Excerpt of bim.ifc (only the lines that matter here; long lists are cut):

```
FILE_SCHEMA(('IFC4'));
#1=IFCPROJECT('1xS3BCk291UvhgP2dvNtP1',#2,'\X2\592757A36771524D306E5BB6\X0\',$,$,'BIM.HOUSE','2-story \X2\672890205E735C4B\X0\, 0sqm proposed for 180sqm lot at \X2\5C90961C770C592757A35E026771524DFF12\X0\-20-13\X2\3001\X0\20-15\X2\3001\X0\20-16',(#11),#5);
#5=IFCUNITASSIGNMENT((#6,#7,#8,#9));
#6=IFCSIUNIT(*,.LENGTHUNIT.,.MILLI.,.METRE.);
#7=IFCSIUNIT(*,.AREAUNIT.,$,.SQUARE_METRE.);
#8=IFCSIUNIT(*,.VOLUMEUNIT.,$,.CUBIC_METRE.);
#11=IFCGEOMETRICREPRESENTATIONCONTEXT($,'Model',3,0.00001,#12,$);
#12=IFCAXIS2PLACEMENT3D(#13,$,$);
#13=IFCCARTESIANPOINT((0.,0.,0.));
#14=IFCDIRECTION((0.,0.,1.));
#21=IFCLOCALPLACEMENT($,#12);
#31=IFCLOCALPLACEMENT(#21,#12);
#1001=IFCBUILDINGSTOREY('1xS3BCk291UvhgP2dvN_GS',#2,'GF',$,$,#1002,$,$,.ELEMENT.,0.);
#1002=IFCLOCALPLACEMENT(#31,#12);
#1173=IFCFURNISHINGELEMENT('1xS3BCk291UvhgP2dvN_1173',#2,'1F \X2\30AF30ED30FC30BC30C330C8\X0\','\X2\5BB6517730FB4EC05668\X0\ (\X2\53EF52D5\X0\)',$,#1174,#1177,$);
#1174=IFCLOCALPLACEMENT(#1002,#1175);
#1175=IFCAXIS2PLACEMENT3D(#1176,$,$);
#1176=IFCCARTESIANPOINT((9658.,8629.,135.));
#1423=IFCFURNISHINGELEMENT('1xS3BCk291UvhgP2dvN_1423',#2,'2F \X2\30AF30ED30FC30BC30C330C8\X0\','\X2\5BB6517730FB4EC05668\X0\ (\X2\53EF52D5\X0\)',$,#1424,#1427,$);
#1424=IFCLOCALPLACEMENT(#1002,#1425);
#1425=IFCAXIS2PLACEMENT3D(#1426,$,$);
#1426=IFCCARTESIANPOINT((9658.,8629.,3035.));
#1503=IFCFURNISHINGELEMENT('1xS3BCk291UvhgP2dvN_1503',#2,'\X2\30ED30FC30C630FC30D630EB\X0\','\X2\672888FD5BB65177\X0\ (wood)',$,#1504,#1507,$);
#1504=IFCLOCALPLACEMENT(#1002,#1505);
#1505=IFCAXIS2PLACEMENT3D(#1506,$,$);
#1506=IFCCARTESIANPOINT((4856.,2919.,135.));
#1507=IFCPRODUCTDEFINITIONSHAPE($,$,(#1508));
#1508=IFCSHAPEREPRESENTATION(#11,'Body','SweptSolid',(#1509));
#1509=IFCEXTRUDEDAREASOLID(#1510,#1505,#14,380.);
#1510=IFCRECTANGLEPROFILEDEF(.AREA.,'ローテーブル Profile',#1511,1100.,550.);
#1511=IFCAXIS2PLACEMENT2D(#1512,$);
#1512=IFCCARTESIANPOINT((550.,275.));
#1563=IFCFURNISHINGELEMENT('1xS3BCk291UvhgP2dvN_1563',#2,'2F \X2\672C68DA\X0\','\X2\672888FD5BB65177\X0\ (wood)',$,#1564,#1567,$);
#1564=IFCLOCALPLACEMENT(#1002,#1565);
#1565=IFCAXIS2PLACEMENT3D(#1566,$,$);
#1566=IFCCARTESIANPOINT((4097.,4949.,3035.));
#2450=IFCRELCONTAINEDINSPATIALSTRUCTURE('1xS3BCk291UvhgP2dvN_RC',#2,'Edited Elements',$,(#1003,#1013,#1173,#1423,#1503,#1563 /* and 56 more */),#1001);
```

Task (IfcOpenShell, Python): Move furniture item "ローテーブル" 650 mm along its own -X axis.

```python
import ifcopenshell
import ifcopenshell.api.geometry
import ifcopenshell.util.placement
import ifcopenshell.util.unit

model = ifcopenshell.open("bim.ifc")
unit_scale = ifcopenshell.util.unit.calculate_unit_scale(model)

item = model.by_id(1503)
matrix = ifcopenshell.util.placement.get_local_placement(item.ObjectPlacement)
matrix[:3, 3] -= matrix[:3, 0] * 0.65 / unit_scale
ifcopenshell.api.geometry.edit_object_placement(model, product=item, matrix=matrix, is_si=False)

print(ifcopenshell.util.placement.get_local_placement(item.ObjectPlacement).round(3) + 0.0)

model.write("bim-out.ifc")
```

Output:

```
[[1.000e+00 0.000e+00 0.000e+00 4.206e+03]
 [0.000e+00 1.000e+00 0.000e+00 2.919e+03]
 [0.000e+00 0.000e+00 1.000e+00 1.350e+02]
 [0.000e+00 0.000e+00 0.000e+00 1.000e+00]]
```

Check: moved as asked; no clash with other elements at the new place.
